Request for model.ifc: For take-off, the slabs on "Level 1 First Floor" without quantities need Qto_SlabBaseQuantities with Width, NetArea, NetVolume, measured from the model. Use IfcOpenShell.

First a look at what the model holds.

```python
import ifcopenshell
import ifcopenshell.util.element
import ifcopenshell.util.unit

model = ifcopenshell.open("model.ifc")
print(model.schema)
for unit_type in ("LENGTHUNIT", "AREAUNIT", "VOLUMEUNIT"):
    print(unit_type, ifcopenshell.util.unit.calculate_unit_scale(model, unit_type))
storey = next(s for s in model.by_type("IfcBuildingStorey") if s.Name == "Level 1 First Floor")
slabs = [e for e in ifcopenshell.util.element.get_decomposition(storey) if e.is_a("IfcSlab")]
for e in sorted(slabs, key=lambda e: e.id()):
    print(e.id(), e.is_a(), e.Name, list(ifcopenshell.util.element.get_psets(e, qtos_only=True)), sep=" | ")
```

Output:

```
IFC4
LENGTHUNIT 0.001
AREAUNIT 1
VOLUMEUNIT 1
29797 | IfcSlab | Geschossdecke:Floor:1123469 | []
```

```python
import ifcopenshell
import ifcopenshell.api.pset
import ifcopenshell.geom
import ifcopenshell.util.element
import ifcopenshell.util.shape
import ifcopenshell.util.unit

model = ifcopenshell.open("model.ifc")
unit_scale = ifcopenshell.util.unit.calculate_unit_scale(model)
area_scale = ifcopenshell.util.unit.calculate_unit_scale(model, "AREAUNIT")
volume_scale = ifcopenshell.util.unit.calculate_unit_scale(model, "VOLUMEUNIT")
settings = ifcopenshell.geom.settings()

storey = next(s for s in model.by_type("IfcBuildingStorey") if s.Name == "Level 1 First Floor")
slabs = [e for e in ifcopenshell.util.element.get_decomposition(storey) if e.is_a("IfcSlab")]

for e in sorted(slabs, key=lambda e: e.id()):
    if ifcopenshell.util.element.get_psets(e, qtos_only=True, should_inherit=False):
        continue
    # Geometry comes back in metres, in the element's own axes.
    shape = ifcopenshell.geom.create_shape(settings, e)
    values = {
        "Width": ifcopenshell.util.shape.get_z(shape.geometry) / unit_scale,
        "NetArea": ifcopenshell.util.shape.get_footprint_area(shape.geometry) / area_scale,
        "NetVolume": ifcopenshell.util.shape.get_volume(shape.geometry) / volume_scale,
    }
    qto = ifcopenshell.api.pset.add_qto(model, product=e, name="Qto_SlabBaseQuantities")
    ifcopenshell.api.pset.edit_qto(model, qto=qto, properties=values)
    print(e.id(), {k: round(v, 3) for k, v in values.items()})

model.write("model_edited.ifc")
```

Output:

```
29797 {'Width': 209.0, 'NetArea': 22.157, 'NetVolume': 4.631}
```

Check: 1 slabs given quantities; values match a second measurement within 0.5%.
